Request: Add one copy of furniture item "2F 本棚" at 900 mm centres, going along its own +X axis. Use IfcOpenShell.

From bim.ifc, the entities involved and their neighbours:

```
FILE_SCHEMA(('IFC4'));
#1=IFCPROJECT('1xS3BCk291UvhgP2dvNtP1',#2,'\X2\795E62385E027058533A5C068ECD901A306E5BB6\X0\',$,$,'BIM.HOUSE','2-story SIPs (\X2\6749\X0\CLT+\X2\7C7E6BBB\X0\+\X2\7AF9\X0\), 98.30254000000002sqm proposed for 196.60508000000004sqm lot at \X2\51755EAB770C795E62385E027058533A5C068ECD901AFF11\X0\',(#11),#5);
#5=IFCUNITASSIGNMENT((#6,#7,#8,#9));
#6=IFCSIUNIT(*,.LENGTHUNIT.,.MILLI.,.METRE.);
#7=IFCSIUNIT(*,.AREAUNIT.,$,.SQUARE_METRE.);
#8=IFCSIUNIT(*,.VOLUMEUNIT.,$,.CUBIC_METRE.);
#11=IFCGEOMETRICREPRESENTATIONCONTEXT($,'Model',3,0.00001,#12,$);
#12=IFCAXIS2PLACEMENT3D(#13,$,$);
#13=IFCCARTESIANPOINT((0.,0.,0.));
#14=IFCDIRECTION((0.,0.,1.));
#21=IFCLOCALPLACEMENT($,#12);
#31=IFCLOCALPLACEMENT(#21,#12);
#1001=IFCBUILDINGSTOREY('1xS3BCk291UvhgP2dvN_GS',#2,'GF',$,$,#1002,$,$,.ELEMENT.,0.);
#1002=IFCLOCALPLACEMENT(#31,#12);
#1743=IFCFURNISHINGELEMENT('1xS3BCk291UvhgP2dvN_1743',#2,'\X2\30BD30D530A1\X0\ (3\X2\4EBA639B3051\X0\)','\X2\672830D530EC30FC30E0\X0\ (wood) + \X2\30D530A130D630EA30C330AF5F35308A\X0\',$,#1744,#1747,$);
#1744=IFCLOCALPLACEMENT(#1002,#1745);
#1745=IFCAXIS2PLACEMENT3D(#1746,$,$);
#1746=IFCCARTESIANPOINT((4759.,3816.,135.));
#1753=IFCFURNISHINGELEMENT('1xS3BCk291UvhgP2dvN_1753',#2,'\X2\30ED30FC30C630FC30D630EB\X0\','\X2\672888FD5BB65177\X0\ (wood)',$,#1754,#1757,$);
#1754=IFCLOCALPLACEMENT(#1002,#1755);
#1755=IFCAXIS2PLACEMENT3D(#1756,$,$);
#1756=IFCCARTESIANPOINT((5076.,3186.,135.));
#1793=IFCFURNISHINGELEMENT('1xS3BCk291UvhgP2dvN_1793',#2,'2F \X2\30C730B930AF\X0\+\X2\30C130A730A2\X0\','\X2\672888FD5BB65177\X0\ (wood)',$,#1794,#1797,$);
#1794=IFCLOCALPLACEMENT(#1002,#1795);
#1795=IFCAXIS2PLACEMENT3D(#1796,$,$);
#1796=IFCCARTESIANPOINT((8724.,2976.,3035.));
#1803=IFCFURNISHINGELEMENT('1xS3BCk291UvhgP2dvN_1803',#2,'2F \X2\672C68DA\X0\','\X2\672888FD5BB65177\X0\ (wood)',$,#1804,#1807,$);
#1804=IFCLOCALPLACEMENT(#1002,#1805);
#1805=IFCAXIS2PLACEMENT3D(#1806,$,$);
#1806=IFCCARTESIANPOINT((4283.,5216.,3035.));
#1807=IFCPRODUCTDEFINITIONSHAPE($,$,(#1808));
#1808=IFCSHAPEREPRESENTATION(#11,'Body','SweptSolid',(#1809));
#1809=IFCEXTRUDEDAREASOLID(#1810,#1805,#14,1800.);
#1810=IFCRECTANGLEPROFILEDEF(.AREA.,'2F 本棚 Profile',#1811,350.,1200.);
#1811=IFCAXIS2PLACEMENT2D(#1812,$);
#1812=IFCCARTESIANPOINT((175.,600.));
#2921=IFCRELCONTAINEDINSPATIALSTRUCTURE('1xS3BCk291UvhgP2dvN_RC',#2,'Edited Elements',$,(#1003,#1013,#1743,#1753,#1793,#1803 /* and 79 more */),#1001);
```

```python
import ifcopenshell
import ifcopenshell.api.geometry
import ifcopenshell.api.root
import ifcopenshell.util.element
import ifcopenshell.util.placement

model = ifcopenshell.open("bim.ifc")


def reuse_history(source, copy):
    """copy_class also copies each property set's owner history, people and application; keep the originals."""
    for rel in copy.IsDefinedBy:
        if rel.is_a("IfcRelDefinesByProperties") and (history := rel.RelatingPropertyDefinition.OwnerHistory):
            rel.RelatingPropertyDefinition.OwnerHistory = source.OwnerHistory
            ifcopenshell.util.element.remove_deep2(model, history)


source = model.by_id(1803)
base = ifcopenshell.util.placement.get_local_placement(source.ObjectPlacement)
step = base[:3, 0] * 900.0

for i in range(1, 2):
    copy = ifcopenshell.api.root.copy_class(model, product=source)
    copy.Representation = ifcopenshell.util.element.copy_deep(
        model, source.Representation, exclude=["IfcGeometricRepresentationContext", "IfcRepresentationMap"]
    )
    reuse_history(source, copy)
    matrix = base.copy()
    matrix[:3, 3] += i * step
    print("added at", matrix[:3, 3].round(3) + 0.0)
    ifcopenshell.api.geometry.edit_object_placement(model, product=copy, matrix=matrix, is_si=False)

model.write("bim-out.ifc")
```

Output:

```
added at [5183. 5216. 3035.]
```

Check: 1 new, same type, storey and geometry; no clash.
